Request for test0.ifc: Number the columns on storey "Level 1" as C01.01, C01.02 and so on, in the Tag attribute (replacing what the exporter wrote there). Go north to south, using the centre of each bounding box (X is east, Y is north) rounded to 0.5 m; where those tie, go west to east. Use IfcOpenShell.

First a look at what the model holds.

```python
import ifcopenshell
import ifcopenshell.util.element
import ifcopenshell.util.placement

model = ifcopenshell.open("test0.ifc")
print(model.schema)
storey = next(s for s in model.by_type("IfcBuildingStorey") if s.Name == "Level 1")
columns = [e for e in ifcopenshell.util.element.get_decomposition(storey) if e.is_a("IfcColumn")]
for e in sorted(columns, key=lambda e: e.id()):
    origin = ifcopenshell.util.placement.get_local_placement(e.ObjectPlacement)[:3, 3]
    print(e.id(), e.Tag, e.Name, origin.round(2) + 0.0, sep=" | ")
```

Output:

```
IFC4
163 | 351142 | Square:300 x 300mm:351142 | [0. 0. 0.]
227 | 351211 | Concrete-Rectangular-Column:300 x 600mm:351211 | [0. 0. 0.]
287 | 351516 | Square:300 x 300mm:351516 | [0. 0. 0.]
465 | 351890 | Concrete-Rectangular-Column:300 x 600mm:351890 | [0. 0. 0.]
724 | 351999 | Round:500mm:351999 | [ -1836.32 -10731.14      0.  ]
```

```python
import ifcopenshell
import ifcopenshell.geom
import ifcopenshell.util.element
import ifcopenshell.util.shape

model = ifcopenshell.open("test0.ifc")
settings = ifcopenshell.geom.settings()
settings.set("use-world-coords", True)


def centre(element):
    shape = ifcopenshell.geom.create_shape(settings, element)
    return ifcopenshell.util.shape.get_bbox_centroid(shape.geometry)


storey = next(s for s in model.by_type("IfcBuildingStorey") if s.Name == "Level 1")
columns = [e for e in ifcopenshell.util.element.get_decomposition(storey) if e.is_a("IfcColumn")]

# Insertion points can sit at a corner or the storey origin, so sort by the geometry (in metres).
centres = {e: centre(e) for e in columns}
columns.sort(key=lambda e: (-round(centres[e][1] / 0.5), centres[e][0]))

for i, e in enumerate(columns, start=1):
    number = f"C01.{i:02d}"
    e.Tag = number
    print(e.id(), number)

model.write("test0_updated.ifc")
```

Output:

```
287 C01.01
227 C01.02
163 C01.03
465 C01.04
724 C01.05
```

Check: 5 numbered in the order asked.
